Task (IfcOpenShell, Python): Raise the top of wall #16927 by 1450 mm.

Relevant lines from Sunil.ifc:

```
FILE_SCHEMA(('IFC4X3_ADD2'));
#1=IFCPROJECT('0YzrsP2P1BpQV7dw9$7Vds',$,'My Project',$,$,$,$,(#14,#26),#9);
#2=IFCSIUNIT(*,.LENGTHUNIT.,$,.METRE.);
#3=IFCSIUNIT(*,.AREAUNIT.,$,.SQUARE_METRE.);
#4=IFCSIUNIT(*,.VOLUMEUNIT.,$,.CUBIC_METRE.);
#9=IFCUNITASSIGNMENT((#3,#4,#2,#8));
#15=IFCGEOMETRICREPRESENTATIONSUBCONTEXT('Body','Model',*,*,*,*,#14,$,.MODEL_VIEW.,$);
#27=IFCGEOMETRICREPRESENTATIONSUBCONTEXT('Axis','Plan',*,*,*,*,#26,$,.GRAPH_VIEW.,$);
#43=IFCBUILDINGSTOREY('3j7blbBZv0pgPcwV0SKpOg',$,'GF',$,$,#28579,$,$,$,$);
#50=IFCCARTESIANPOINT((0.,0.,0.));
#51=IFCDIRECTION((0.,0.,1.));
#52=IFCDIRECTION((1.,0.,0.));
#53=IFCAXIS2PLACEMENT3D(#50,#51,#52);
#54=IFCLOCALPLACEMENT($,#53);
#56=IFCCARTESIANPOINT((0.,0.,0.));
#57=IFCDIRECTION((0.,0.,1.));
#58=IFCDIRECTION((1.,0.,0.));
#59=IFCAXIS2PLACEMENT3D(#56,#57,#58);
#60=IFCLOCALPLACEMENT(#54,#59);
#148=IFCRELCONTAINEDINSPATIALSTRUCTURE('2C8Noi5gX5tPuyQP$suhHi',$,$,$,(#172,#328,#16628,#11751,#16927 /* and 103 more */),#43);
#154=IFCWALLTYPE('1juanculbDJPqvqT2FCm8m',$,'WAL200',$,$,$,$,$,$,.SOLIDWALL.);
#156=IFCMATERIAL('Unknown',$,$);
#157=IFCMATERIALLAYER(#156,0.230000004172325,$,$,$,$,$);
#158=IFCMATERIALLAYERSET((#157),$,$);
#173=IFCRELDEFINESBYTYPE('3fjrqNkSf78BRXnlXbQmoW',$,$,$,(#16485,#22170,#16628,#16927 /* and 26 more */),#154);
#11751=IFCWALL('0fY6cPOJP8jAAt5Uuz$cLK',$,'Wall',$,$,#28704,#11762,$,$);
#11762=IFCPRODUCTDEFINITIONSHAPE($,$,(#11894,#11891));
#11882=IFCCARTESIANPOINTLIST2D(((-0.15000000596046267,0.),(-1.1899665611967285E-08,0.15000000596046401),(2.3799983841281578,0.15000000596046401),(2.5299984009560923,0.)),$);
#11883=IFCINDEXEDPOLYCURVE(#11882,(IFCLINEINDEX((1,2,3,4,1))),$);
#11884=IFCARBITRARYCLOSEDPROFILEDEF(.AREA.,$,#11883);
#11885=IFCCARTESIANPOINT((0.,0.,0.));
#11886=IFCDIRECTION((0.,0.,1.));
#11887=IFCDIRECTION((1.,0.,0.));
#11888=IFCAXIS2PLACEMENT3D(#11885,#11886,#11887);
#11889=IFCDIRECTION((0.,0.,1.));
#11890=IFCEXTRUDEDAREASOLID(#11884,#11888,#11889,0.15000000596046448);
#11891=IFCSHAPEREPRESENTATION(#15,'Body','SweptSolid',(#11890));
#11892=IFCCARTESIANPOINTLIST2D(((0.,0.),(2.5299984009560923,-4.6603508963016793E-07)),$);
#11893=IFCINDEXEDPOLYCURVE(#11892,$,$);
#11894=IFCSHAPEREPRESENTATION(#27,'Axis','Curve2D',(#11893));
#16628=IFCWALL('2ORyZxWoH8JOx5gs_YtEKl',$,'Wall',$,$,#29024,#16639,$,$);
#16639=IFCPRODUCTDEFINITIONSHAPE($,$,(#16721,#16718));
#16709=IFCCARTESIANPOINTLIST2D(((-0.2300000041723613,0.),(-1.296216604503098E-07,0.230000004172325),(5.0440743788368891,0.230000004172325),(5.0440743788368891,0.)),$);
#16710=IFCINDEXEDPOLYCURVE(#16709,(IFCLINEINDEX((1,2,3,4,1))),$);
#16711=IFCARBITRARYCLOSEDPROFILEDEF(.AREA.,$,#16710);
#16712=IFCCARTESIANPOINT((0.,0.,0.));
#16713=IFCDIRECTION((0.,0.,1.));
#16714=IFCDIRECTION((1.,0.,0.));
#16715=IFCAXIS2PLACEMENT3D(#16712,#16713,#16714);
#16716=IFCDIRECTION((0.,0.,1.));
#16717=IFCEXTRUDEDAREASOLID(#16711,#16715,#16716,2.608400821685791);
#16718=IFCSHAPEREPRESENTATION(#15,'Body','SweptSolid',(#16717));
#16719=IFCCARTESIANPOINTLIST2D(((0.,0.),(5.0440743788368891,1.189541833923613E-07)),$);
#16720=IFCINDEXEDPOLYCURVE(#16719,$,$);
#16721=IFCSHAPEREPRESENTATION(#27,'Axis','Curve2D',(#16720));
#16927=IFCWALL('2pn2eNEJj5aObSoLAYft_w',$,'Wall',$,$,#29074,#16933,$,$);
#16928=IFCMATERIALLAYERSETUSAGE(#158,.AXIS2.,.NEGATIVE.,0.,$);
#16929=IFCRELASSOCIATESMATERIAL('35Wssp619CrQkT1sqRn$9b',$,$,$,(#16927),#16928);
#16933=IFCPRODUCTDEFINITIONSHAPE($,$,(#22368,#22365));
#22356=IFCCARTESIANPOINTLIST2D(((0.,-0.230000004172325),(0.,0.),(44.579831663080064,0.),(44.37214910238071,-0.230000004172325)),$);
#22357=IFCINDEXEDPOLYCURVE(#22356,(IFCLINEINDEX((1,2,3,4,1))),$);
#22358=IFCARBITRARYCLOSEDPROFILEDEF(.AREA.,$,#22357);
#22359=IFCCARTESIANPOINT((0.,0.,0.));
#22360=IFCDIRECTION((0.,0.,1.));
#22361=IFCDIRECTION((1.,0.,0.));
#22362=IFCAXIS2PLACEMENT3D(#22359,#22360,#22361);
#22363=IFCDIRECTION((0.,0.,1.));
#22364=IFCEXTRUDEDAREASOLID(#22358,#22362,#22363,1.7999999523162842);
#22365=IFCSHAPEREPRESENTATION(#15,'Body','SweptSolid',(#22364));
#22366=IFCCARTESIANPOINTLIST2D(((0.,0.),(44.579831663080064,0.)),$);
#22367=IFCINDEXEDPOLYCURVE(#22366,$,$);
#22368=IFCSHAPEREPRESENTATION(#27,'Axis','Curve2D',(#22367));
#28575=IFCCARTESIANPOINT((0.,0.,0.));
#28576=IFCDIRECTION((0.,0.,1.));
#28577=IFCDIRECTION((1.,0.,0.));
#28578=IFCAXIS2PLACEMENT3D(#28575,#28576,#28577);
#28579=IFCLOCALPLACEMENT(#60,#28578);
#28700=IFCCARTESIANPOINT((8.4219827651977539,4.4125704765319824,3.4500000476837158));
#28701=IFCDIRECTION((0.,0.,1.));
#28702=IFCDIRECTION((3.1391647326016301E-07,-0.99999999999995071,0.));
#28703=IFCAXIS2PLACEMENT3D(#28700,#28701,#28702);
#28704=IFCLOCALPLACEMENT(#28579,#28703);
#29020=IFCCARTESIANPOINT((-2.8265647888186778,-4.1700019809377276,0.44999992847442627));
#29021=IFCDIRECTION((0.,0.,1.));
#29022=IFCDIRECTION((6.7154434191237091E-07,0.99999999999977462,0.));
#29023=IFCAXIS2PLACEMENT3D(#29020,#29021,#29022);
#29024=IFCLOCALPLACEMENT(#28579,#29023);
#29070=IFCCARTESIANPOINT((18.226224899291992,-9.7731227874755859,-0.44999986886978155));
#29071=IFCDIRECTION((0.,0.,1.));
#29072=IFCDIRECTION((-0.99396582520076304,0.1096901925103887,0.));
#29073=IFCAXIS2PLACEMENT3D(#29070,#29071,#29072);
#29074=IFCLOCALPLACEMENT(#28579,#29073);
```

```python
import ifcopenshell
import ifcopenshell.geom
import ifcopenshell.util.representation
import ifcopenshell.util.shape
import ifcopenshell.util.unit

model = ifcopenshell.open("Sunil.ifc")
unit_scale = ifcopenshell.util.unit.calculate_unit_scale(model)
settings = ifcopenshell.geom.settings()


def volume(element):
    """Net volume in cubic metres, openings subtracted."""
    shape = ifcopenshell.geom.create_shape(settings, element)
    return ifcopenshell.util.shape.get_volume(shape.geometry)


wall = model.by_id(16927)
before = volume(wall)

body = ifcopenshell.util.representation.get_representation(wall, "Model", "Body")
solid = body.Items[0]
old_height = solid.Depth
solid.Depth += 1.45 / unit_scale
after = volume(wall)

print(f"height {old_height:g} -> {solid.Depth:g}, volume {before:.3f} -> {after:.3f} m3")

model.write("Sunil-out.ifc")
```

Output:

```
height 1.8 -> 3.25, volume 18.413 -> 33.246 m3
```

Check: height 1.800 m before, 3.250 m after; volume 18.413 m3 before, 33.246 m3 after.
